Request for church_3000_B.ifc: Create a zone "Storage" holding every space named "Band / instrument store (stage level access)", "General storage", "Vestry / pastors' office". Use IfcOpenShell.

First a look at what the model holds.

```python
import ifcopenshell

model = ifcopenshell.open("church_3000_B.ifc")
print(model.schema)
seen = {}
for space in model.by_type("IfcSpace"):
    seen[space.LongName] = seen.get(space.LongName, 0) + 1
for name, count in sorted(seen.items(), key=str):
    print(count, "x", name)
print("zones:", [z.Name for z in model.by_type("IfcZone")][:20])
```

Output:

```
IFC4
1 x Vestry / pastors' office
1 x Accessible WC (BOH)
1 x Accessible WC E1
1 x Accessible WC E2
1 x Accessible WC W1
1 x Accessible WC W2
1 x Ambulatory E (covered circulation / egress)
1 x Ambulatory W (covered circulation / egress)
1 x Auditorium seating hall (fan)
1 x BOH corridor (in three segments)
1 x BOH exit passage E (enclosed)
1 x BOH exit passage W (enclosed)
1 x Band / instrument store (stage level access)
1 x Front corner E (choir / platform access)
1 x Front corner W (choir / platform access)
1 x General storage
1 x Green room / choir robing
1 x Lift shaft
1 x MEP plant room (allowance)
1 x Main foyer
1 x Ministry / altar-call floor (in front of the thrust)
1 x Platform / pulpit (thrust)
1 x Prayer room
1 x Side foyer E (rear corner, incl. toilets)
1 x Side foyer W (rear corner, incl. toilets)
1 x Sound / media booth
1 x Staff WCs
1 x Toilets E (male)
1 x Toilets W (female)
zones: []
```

```python
import ifcopenshell
import ifcopenshell.api.group
import ifcopenshell.api.root

model = ifcopenshell.open("church_3000_B.ifc")

names = {"Band / instrument store (stage level access)", "General storage", "Vestry / pastors' office"}
spaces = [s for s in model.by_type("IfcSpace") if s.LongName in names]

zone = ifcopenshell.api.root.create_entity(model, ifc_class="IfcZone", name="Storage")
ifcopenshell.api.group.assign_group(model, products=spaces, group=zone)
print(len(spaces), "spaces in", zone.Name)

model.write("church_3000_B_edited.ifc")
```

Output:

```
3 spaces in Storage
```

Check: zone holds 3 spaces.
